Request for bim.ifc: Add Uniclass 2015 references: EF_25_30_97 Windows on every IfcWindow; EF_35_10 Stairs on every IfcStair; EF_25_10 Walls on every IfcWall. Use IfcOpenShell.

First a look at what the model holds.

```python
import ifcopenshell

model = ifcopenshell.open("bim.ifc")
print(model.schema)
print("classifications:", [c.Name for c in model.by_type("IfcClassification")])
for ifc_class in ("IfcDoor", "IfcRoof", "IfcStair", "IfcWall", "IfcWindow"):
    print(ifc_class, len(model.by_type(ifc_class)))
```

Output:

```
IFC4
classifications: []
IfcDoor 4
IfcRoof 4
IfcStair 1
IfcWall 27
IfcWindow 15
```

```python
import ifcopenshell
import ifcopenshell.api.classification

model = ifcopenshell.open("bim.ifc")

system = ifcopenshell.api.classification.add_classification(model, classification="Uniclass 2015")

codes = {
    "IfcWindow": ("EF_25_30_97", "Windows"),
    "IfcStair": ("EF_35_10", "Stairs"),
    "IfcWall": ("EF_25_10", "Walls"),
}
for ifc_class, (code, name) in codes.items():
    products = model.by_type(ifc_class)
    ifcopenshell.api.classification.add_reference(
        model, products=products, classification=system, identification=code, name=name
    )
    print(code, len(products))

model.write("bim-out.ifc")
```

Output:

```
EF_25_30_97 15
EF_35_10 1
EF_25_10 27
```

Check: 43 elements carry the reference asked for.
